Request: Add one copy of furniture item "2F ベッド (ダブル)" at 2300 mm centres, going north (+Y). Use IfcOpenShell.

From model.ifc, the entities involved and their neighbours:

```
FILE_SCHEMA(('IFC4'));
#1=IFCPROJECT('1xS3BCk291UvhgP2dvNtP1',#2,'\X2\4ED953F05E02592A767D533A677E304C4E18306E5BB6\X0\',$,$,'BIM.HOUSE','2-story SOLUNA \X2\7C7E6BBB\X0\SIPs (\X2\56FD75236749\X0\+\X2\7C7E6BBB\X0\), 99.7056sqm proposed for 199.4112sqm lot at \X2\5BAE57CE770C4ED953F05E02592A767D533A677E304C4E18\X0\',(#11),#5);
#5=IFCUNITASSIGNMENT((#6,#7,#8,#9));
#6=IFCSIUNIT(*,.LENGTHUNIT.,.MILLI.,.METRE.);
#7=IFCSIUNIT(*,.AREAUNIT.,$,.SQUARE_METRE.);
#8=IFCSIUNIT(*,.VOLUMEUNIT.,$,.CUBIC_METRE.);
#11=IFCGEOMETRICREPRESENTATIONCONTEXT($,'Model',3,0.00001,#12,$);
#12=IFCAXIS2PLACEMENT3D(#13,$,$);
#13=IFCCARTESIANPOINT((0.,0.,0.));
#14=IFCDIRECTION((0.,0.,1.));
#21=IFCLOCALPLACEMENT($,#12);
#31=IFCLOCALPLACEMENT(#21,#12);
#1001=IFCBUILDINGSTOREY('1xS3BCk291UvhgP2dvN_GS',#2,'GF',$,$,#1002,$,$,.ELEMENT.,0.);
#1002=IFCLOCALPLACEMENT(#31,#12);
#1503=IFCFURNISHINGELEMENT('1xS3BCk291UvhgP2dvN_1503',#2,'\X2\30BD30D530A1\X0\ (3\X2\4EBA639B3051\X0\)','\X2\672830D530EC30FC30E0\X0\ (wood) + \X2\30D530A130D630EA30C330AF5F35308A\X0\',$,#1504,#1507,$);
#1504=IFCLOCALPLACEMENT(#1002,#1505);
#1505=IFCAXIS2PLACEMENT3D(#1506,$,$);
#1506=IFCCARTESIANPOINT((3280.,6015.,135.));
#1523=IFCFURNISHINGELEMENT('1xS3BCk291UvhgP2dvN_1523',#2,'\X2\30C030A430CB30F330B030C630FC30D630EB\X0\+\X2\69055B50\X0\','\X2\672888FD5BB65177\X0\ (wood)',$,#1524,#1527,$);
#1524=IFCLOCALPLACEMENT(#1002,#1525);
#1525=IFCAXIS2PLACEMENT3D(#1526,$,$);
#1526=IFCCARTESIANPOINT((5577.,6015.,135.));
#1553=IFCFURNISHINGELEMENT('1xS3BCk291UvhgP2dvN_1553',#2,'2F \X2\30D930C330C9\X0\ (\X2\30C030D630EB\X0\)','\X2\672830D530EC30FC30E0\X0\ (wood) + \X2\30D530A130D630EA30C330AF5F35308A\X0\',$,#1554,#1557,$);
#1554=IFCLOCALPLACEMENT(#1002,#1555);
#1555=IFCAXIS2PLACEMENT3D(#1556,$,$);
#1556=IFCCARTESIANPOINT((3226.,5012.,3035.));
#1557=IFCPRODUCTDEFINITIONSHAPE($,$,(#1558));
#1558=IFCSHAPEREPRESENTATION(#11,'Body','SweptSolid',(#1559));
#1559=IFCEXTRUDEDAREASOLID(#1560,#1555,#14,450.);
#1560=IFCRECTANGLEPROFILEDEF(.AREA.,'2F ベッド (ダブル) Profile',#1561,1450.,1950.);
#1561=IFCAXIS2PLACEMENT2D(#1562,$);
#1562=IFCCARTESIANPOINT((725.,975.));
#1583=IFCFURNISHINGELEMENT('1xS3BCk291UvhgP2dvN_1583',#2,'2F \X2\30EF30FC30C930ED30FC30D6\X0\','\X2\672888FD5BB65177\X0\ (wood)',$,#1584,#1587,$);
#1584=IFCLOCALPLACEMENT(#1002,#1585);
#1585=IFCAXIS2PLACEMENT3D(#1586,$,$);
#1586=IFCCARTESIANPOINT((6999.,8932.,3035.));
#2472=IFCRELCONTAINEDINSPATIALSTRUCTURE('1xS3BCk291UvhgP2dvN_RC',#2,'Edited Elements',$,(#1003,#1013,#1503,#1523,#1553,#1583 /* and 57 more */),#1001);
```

```python
import numpy as np
import ifcopenshell
import ifcopenshell.api.geometry
import ifcopenshell.api.root
import ifcopenshell.util.element
import ifcopenshell.util.placement
import ifcopenshell.util.unit

model = ifcopenshell.open("model.ifc")
unit_scale = ifcopenshell.util.unit.calculate_unit_scale(model)


def reuse_history(source, copy):
    """copy_class also copies each property set's owner history, people and application; keep the originals."""
    for rel in copy.IsDefinedBy:
        if rel.is_a("IfcRelDefinesByProperties") and (history := rel.RelatingPropertyDefinition.OwnerHistory):
            rel.RelatingPropertyDefinition.OwnerHistory = source.OwnerHistory
            ifcopenshell.util.element.remove_deep2(model, history)


source = model.by_guid("1xS3BCk291UvhgP2dvN_1553")
base = ifcopenshell.util.placement.get_local_placement(source.ObjectPlacement)
step = np.array([0.0, 1.0, 0.0]) * 2.3 / unit_scale

for i in range(1, 2):
    copy = ifcopenshell.api.root.copy_class(model, product=source)
    copy.Representation = ifcopenshell.util.element.copy_deep(
        model, source.Representation, exclude=["IfcGeometricRepresentationContext", "IfcRepresentationMap"]
    )
    reuse_history(source, copy)
    matrix = base.copy()
    matrix[:3, 3] += i * step
    print("added at", matrix[:3, 3].round(3) + 0.0)
    ifcopenshell.api.geometry.edit_object_placement(model, product=copy, matrix=matrix, is_si=False)

model.write("model_rev.ifc")
```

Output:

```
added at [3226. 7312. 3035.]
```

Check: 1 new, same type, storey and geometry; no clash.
